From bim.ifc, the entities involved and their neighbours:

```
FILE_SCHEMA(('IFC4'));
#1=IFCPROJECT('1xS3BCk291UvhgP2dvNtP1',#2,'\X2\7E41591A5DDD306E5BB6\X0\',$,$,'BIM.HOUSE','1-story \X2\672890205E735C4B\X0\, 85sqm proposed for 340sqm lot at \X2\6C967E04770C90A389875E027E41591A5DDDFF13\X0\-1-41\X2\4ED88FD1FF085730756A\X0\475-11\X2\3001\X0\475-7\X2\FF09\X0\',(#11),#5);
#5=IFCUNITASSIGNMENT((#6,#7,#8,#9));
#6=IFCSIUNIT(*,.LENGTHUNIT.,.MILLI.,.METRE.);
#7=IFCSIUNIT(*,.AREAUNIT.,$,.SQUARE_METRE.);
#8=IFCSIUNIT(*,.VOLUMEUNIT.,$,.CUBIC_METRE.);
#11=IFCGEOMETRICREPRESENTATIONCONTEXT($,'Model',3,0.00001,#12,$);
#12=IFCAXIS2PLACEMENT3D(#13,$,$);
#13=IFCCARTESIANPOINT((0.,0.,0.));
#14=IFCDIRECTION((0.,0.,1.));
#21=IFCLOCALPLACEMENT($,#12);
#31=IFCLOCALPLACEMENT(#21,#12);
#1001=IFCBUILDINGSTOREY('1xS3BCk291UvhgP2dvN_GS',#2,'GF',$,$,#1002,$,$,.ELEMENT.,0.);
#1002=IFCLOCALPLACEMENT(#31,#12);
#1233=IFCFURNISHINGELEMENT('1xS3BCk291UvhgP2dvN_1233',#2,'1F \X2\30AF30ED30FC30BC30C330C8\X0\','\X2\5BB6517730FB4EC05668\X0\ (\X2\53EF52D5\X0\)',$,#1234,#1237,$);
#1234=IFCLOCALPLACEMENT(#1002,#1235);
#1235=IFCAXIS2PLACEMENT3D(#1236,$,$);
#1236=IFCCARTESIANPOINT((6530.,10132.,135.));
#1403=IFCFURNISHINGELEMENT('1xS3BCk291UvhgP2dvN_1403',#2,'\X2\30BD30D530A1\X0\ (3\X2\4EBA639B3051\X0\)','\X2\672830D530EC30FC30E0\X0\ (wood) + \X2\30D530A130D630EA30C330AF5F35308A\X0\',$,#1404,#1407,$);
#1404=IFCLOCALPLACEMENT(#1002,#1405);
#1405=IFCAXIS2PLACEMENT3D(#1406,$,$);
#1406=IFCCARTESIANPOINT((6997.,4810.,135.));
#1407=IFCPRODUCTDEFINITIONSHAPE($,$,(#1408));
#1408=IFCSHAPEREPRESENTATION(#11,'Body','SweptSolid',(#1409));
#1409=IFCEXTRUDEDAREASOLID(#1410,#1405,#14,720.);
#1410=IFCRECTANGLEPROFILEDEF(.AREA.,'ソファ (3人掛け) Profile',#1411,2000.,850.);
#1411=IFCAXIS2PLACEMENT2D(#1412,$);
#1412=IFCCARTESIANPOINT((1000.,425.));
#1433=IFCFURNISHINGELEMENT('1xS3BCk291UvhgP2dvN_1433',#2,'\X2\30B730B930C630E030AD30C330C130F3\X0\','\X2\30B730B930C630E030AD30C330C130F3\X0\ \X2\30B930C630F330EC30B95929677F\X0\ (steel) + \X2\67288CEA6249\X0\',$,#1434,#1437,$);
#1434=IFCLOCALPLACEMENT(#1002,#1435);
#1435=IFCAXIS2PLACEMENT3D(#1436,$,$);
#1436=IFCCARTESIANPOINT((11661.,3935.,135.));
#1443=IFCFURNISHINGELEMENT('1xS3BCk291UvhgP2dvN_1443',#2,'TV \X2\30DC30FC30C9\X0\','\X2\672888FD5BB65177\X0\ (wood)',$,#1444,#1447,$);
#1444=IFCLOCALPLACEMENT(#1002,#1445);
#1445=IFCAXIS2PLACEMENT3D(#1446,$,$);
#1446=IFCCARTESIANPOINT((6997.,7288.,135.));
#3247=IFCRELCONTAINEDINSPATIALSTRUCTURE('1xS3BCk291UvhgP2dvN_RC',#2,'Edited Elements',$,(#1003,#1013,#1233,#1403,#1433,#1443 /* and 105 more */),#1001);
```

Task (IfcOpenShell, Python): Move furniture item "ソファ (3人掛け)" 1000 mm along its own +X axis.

```python
import ifcopenshell
import ifcopenshell.api.geometry
import ifcopenshell.util.placement
import ifcopenshell.util.unit

model = ifcopenshell.open("bim.ifc")
unit_scale = ifcopenshell.util.unit.calculate_unit_scale(model)

item = model.by_guid("1xS3BCk291UvhgP2dvN_1403")
matrix = ifcopenshell.util.placement.get_local_placement(item.ObjectPlacement)
matrix[:3, 3] += matrix[:3, 0] * 1 / unit_scale
ifcopenshell.api.geometry.edit_object_placement(model, product=item, matrix=matrix, is_si=False)

print(ifcopenshell.util.placement.get_local_placement(item.ObjectPlacement).round(3) + 0.0)

model.write("bim-out.ifc")
```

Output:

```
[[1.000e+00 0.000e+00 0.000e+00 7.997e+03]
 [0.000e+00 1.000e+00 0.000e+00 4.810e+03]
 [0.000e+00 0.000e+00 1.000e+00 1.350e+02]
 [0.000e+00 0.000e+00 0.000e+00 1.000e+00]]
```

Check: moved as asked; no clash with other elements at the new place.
